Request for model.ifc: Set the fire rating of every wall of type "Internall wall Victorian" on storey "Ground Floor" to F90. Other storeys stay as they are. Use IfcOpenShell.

First a look at what the model holds.

```python
import ifcopenshell
import ifcopenshell.util.element

model = ifcopenshell.open("model.ifc")
print(model.schema)
storey = next(s for s in model.by_type("IfcBuildingStorey") if s.Name == "Ground Floor")
walls = [e for e in ifcopenshell.util.element.get_decomposition(storey) if e.is_a("IfcWall")]
seen = {}
for e in walls:
    element_type = ifcopenshell.util.element.get_type(e)
    key = (element_type.Name if element_type != e and element_type else None, ifcopenshell.util.element.get_pset(e, "Pset_WallCommon", "FireRating"))
    seen[key] = seen.get(key, 0) + 1
for (name, value), count in sorted(seen.items(), key=str):
    print(count, "x", name, "|", value)
```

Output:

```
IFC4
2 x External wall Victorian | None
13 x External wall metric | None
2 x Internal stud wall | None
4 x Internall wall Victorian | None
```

```python
import ifcopenshell
import ifcopenshell.api.pset
import ifcopenshell.util.element

model = ifcopenshell.open("model.ifc")

storey = next(s for s in model.by_type("IfcBuildingStorey") if s.Name == "Ground Floor")
walls = [e for e in ifcopenshell.util.element.get_decomposition(storey) if e.is_a("IfcWall")]

count = 0
for e in walls:
    element_type = ifcopenshell.util.element.get_type(e)
    if element_type in (None, e) or element_type.Name != "Internall wall Victorian":
        continue
    # add_pset returns the element's existing set when there is one.
    pset = ifcopenshell.api.pset.add_pset(model, product=e, name="Pset_WallCommon")
    ifcopenshell.api.pset.edit_pset(model, pset=pset, properties={"FireRating": "F90"})
    count += 1

print(count, "walls updated")

model.write("model_edited.ifc")
```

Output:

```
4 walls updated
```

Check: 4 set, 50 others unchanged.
